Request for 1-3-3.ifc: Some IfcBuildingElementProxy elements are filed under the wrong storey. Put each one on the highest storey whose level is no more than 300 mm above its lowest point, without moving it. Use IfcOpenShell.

First a look at what the model holds.

```python
import ifcopenshell
import ifcopenshell.util.element
import ifcopenshell.util.placement

model = ifcopenshell.open("1-3-3.ifc")
print(model.schema)
for storey in model.by_type("IfcBuildingStorey"):
    level = ifcopenshell.util.placement.get_storey_elevation(storey)
    count = sum(e.is_a("IfcBuildingElementProxy") for e in ifcopenshell.util.element.get_contained(storey))
    print(storey.id(), storey.Name, round(level, 3), count, sep=" | ")
```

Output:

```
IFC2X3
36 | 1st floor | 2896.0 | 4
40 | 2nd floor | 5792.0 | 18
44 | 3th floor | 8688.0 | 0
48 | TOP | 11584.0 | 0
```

```python
import ifcopenshell
import ifcopenshell.api.spatial
import ifcopenshell.geom
import ifcopenshell.util.element
import ifcopenshell.util.placement
import ifcopenshell.util.shape
import ifcopenshell.util.unit

model = ifcopenshell.open("1-3-3.ifc")
unit_scale = ifcopenshell.util.unit.calculate_unit_scale(model)
settings = ifcopenshell.geom.settings()

levels = sorted(
    ((ifcopenshell.util.placement.get_storey_elevation(s) * unit_scale, s) for s in model.by_type("IfcBuildingStorey")),
    key=lambda pair: pair[0],
)

for e in model.by_type("IfcBuildingElementProxy"):
    current = e.ContainedInStructure[0].RelatingStructure if e.ContainedInStructure else None
    if current is None or not current.is_a("IfcBuildingStorey"):
        continue
    shape = ifcopenshell.geom.create_shape(settings, e)
    bottom = ifcopenshell.util.shape.get_shape_bottom_elevation(shape, shape.geometry)
    below = [s for level, s in levels if level <= bottom + 0.3]
    storey = below[-1] if below else levels[0][1]
    if storey != current:
        # assign_container keeps the world position.
        ifcopenshell.api.spatial.assign_container(model, products=[e], relating_structure=storey)
        print(e.id(), current.Name, "->", storey.Name)

model.write("1-3-3_rev.ifc")
```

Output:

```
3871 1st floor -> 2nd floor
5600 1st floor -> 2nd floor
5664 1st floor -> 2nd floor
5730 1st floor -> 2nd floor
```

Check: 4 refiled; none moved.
